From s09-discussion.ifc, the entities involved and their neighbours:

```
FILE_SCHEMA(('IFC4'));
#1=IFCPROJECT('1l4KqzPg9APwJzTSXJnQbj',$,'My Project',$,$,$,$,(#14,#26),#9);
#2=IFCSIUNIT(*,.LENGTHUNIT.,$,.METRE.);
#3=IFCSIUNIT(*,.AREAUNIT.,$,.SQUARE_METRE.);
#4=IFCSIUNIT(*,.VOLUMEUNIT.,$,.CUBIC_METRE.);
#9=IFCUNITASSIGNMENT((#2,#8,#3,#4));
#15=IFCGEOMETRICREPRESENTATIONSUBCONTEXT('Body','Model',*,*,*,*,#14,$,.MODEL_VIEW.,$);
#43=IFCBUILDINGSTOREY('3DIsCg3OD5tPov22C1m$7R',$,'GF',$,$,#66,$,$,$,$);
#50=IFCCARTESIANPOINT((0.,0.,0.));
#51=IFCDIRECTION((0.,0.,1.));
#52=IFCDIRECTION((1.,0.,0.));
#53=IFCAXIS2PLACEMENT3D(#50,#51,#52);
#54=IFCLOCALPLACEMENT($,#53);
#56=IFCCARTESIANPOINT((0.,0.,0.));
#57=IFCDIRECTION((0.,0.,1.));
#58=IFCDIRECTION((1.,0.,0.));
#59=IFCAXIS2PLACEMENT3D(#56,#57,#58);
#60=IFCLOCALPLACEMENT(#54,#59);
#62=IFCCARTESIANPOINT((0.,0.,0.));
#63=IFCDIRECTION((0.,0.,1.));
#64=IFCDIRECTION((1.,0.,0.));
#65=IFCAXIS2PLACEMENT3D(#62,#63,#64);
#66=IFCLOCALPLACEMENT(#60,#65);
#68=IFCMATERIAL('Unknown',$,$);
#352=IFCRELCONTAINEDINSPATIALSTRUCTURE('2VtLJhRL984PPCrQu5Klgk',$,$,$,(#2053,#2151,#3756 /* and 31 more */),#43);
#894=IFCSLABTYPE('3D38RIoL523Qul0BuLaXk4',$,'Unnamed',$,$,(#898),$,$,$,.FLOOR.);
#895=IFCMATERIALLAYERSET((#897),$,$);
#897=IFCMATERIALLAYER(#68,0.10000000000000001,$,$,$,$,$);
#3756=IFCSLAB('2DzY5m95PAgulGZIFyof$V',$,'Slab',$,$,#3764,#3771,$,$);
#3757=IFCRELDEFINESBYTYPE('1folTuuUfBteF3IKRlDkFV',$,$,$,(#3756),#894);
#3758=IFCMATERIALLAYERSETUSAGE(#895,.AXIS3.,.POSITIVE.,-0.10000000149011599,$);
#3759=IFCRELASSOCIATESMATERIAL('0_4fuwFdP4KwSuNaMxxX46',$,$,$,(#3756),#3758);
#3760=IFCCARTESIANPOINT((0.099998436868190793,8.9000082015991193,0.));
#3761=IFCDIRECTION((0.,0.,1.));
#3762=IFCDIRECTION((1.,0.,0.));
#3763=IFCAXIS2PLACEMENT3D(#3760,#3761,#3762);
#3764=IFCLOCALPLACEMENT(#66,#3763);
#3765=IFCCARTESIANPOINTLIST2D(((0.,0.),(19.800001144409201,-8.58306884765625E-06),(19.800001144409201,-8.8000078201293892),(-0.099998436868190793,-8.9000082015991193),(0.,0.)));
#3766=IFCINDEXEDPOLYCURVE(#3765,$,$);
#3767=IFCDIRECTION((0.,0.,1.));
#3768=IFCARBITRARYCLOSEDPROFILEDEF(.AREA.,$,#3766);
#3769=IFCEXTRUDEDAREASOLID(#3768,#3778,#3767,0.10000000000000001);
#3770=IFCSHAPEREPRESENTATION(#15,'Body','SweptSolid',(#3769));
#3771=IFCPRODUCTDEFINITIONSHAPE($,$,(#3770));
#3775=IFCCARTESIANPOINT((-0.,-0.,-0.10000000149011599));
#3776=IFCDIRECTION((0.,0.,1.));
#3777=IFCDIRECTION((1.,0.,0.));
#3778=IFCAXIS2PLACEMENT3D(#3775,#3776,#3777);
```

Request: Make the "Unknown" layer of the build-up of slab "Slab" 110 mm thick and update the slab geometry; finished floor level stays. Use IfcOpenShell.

```python
import ifcopenshell
import ifcopenshell.util.element
import ifcopenshell.util.representation
import ifcopenshell.util.unit

model = ifcopenshell.open("s09-discussion.ifc")
unit_scale = ifcopenshell.util.unit.calculate_unit_scale(model)

layer_set = model.by_id(895)
layer = next(l for l in layer_set.MaterialLayers if l.Material and l.Material.Name == "Unknown")
change = 0.11 / unit_scale - layer.LayerThickness
layer.LayerThickness += change

# Geometry does not follow the layer set by itself.
slabs = [e for e in ifcopenshell.util.element.get_elements_by_material(model, layer_set) if e.is_a("IfcSlab")]
for slab in sorted(slabs, key=lambda e: e.id()):
    body = ifcopenshell.util.representation.get_representation(slab, "Model", "Body")
    solid = body.Items[0]
    old_depth = solid.Depth
    solid.Depth += change
    # Extruded upwards: lower the start of the extrusion so the top stays.
    x, y, z = solid.Position.Location.Coordinates
    solid.Position.Location = model.createIfcCartesianPoint((x, y, z - change))
    print(slab.id(), f"{old_depth:g} -> {solid.Depth:g}")

# The layers are counted up from the underside, which has moved.
for usage in {ifcopenshell.util.element.get_material(slab) for slab in slabs}:
    usage.OffsetFromReferenceLine -= change

model.write("s09-discussion_v2.ifc")
```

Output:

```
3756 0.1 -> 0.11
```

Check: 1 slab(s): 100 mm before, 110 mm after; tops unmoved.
